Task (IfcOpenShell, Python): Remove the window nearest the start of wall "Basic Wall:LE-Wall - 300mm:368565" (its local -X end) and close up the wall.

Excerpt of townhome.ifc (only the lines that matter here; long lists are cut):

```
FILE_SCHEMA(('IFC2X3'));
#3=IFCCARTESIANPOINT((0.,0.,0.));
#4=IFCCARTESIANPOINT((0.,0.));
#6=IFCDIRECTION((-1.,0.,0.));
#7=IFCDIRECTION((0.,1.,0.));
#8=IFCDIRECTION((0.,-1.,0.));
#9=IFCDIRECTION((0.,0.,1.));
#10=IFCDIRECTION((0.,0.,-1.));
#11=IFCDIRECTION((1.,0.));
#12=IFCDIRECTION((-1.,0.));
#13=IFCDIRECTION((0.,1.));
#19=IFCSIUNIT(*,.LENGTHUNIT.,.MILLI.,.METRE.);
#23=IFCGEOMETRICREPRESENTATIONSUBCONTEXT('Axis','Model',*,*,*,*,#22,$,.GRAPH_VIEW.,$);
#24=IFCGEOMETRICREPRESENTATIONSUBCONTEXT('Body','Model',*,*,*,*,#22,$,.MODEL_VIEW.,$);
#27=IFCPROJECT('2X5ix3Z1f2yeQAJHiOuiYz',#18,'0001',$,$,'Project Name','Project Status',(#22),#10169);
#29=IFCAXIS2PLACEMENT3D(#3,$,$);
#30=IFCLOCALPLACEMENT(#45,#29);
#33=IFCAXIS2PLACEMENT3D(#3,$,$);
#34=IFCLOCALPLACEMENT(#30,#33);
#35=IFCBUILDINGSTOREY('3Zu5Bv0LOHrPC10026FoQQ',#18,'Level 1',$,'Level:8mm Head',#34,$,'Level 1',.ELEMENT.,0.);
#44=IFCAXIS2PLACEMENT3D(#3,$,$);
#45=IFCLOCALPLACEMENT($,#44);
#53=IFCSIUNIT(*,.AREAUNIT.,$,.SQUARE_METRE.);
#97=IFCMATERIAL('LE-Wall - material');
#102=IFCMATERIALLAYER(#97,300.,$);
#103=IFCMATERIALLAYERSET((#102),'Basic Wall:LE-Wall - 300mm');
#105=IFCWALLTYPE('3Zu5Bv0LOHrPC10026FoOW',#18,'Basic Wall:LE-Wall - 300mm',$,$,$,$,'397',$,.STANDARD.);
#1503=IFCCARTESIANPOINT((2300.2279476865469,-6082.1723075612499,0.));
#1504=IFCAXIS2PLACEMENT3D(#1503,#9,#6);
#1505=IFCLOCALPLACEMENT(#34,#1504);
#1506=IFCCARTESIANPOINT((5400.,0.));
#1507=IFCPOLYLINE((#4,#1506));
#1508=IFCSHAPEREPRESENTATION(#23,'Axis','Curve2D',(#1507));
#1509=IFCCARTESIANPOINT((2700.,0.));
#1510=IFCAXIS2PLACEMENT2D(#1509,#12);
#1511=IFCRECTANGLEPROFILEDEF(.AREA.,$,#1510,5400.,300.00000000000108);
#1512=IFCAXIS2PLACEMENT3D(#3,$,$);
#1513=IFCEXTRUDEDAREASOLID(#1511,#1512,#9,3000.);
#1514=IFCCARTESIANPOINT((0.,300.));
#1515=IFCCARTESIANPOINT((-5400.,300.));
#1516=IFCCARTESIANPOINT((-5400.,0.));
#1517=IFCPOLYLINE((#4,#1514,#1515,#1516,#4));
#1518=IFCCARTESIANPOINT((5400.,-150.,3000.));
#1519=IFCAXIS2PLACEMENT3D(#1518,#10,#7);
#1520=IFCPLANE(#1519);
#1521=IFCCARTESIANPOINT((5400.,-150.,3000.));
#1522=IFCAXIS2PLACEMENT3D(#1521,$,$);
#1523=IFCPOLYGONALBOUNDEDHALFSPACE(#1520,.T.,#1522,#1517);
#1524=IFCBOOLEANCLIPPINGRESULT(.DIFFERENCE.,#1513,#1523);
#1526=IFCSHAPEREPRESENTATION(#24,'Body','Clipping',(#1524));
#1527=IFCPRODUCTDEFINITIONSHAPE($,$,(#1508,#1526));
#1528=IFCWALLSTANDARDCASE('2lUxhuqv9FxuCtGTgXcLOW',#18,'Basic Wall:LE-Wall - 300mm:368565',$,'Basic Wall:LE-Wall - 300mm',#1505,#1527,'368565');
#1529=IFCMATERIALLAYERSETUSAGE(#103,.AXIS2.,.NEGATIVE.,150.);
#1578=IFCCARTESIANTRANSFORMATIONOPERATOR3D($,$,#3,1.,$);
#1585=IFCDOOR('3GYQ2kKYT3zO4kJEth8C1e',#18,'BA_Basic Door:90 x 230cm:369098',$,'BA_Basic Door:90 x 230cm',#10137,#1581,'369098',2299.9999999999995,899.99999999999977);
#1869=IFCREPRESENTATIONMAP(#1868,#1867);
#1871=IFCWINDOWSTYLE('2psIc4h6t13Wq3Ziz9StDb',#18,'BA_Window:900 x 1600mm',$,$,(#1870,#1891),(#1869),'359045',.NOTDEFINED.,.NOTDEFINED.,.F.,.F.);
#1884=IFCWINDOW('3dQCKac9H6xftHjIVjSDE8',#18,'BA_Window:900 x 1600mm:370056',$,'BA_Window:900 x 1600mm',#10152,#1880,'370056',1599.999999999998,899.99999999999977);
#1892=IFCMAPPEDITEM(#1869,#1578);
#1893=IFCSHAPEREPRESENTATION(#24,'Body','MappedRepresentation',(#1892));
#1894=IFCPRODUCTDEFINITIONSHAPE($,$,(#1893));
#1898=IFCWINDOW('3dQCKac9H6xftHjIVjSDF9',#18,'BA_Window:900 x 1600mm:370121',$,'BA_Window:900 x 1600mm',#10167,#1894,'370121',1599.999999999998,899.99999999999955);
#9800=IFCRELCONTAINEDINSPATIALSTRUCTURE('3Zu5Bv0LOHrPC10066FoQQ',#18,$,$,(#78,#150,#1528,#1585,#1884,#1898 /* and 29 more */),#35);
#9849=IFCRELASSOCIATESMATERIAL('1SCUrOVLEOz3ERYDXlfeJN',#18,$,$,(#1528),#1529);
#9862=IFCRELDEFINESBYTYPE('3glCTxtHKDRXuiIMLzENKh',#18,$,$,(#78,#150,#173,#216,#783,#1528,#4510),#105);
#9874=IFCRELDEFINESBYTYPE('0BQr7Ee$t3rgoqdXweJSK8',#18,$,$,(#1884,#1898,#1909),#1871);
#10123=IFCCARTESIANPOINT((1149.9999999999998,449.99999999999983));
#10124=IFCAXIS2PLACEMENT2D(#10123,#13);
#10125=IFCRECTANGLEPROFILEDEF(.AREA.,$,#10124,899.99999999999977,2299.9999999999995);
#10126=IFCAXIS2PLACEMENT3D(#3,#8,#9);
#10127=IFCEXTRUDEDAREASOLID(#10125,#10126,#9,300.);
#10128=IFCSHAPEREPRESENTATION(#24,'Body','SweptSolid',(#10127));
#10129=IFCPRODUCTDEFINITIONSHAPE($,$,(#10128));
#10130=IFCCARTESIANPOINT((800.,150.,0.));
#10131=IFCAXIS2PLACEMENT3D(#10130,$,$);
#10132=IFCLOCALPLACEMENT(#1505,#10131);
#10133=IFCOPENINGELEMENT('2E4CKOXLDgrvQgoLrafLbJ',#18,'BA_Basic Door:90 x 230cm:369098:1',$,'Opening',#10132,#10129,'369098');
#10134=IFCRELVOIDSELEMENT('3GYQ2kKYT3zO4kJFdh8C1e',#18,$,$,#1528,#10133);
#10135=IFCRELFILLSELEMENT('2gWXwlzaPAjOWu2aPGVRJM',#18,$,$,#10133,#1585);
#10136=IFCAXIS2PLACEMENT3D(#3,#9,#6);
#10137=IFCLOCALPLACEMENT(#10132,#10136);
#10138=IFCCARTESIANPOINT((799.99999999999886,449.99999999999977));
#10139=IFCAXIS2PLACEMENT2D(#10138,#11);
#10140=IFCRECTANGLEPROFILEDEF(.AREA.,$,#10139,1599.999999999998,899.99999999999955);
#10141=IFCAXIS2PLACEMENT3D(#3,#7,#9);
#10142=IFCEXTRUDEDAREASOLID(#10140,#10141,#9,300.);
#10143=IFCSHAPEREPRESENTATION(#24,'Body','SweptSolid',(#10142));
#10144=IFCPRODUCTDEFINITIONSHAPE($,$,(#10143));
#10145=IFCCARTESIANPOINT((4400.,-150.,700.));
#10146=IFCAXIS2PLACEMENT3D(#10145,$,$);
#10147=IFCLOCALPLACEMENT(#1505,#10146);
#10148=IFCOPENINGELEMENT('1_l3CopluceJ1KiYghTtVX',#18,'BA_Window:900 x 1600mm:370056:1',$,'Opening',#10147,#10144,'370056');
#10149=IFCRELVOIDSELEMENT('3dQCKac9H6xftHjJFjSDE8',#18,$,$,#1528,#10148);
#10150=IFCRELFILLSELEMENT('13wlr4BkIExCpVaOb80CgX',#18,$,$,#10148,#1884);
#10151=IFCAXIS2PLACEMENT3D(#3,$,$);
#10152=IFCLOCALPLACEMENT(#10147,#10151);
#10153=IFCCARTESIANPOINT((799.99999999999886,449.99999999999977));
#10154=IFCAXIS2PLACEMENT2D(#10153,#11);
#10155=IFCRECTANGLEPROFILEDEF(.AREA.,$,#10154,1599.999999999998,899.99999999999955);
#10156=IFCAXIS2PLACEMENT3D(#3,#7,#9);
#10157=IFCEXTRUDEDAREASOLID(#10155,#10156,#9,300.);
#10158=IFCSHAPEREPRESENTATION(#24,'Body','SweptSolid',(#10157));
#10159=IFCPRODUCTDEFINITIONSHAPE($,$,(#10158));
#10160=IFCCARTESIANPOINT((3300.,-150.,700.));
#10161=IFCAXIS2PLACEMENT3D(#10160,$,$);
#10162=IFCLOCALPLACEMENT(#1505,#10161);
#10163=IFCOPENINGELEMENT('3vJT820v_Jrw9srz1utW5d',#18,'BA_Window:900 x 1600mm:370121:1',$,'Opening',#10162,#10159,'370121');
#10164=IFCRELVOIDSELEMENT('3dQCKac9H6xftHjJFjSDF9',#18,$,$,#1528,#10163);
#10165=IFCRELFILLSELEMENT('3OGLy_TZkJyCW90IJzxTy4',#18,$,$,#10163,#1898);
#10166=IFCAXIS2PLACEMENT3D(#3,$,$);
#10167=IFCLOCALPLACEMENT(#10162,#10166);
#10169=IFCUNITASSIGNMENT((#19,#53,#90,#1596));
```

```python
import ifcopenshell
import ifcopenshell.api.feature
import ifcopenshell.api.root
import ifcopenshell.geom
import ifcopenshell.util.shape

model = ifcopenshell.open("townhome.ifc")
settings = ifcopenshell.geom.settings()


def volume(element):
    """Net volume in cubic metres, openings subtracted."""
    shape = ifcopenshell.geom.create_shape(settings, element)
    return ifcopenshell.util.shape.get_volume(shape.geometry)


window = model.by_id(1898)
opening = window.FillsVoids[0].RelatingOpeningElement
wall = opening.VoidsElements[0].RelatingBuildingElement
before = volume(wall)

ifcopenshell.api.root.remove_product(model, product=window)
ifcopenshell.api.feature.remove_feature(model, feature=opening)

after = volume(wall)

print(f"wall volume {before:.3f} -> {after:.3f} m3")

model.write("townhome-out.ifc")
```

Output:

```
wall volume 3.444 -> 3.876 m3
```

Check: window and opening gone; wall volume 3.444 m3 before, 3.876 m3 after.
